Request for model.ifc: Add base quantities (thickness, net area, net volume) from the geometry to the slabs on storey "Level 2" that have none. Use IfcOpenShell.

First a look at what the model holds.

```python
import ifcopenshell
import ifcopenshell.util.element
import ifcopenshell.util.unit

model = ifcopenshell.open("model.ifc")
print(model.schema)
for unit_type in ("LENGTHUNIT", "AREAUNIT", "VOLUMEUNIT"):
    print(unit_type, ifcopenshell.util.unit.calculate_unit_scale(model, unit_type))
storey = next(s for s in model.by_type("IfcBuildingStorey") if s.Name == "Level 2")
slabs = [e for e in ifcopenshell.util.element.get_decomposition(storey) if e.is_a("IfcSlab")]
for e in sorted(slabs, key=lambda e: e.id()):
    print(e.id(), e.is_a(), e.Name, list(ifcopenshell.util.element.get_psets(e, qtos_only=True)), sep=" | ")
```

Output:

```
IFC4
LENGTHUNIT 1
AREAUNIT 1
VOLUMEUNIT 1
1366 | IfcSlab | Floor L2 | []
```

```python
import ifcopenshell
import ifcopenshell.api.pset
import ifcopenshell.geom
import ifcopenshell.util.element
import ifcopenshell.util.shape
import ifcopenshell.util.unit

model = ifcopenshell.open("model.ifc")
unit_scale = ifcopenshell.util.unit.calculate_unit_scale(model)
area_scale = ifcopenshell.util.unit.calculate_unit_scale(model, "AREAUNIT")
volume_scale = ifcopenshell.util.unit.calculate_unit_scale(model, "VOLUMEUNIT")
settings = ifcopenshell.geom.settings()

storey = next(s for s in model.by_type("IfcBuildingStorey") if s.Name == "Level 2")
slabs = [e for e in ifcopenshell.util.element.get_decomposition(storey) if e.is_a("IfcSlab")]

for e in sorted(slabs, key=lambda e: e.id()):
    if ifcopenshell.util.element.get_psets(e, qtos_only=True, should_inherit=False):
        continue
    # Geometry comes back in metres, in the element's own axes.
    shape = ifcopenshell.geom.create_shape(settings, e)
    values = {
        "Width": ifcopenshell.util.shape.get_z(shape.geometry) / unit_scale,
        "NetArea": ifcopenshell.util.shape.get_footprint_area(shape.geometry) / area_scale,
        "NetVolume": ifcopenshell.util.shape.get_volume(shape.geometry) / volume_scale,
    }
    qto = ifcopenshell.api.pset.add_qto(model, product=e, name="Qto_SlabBaseQuantities")
    ifcopenshell.api.pset.edit_qto(model, qto=qto, properties=values)
    print(e.id(), {k: round(v, 3) for k, v in values.items()})

model.write("model_updated.ifc")
```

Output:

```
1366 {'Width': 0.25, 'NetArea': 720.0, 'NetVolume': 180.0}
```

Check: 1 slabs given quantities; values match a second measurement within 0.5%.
